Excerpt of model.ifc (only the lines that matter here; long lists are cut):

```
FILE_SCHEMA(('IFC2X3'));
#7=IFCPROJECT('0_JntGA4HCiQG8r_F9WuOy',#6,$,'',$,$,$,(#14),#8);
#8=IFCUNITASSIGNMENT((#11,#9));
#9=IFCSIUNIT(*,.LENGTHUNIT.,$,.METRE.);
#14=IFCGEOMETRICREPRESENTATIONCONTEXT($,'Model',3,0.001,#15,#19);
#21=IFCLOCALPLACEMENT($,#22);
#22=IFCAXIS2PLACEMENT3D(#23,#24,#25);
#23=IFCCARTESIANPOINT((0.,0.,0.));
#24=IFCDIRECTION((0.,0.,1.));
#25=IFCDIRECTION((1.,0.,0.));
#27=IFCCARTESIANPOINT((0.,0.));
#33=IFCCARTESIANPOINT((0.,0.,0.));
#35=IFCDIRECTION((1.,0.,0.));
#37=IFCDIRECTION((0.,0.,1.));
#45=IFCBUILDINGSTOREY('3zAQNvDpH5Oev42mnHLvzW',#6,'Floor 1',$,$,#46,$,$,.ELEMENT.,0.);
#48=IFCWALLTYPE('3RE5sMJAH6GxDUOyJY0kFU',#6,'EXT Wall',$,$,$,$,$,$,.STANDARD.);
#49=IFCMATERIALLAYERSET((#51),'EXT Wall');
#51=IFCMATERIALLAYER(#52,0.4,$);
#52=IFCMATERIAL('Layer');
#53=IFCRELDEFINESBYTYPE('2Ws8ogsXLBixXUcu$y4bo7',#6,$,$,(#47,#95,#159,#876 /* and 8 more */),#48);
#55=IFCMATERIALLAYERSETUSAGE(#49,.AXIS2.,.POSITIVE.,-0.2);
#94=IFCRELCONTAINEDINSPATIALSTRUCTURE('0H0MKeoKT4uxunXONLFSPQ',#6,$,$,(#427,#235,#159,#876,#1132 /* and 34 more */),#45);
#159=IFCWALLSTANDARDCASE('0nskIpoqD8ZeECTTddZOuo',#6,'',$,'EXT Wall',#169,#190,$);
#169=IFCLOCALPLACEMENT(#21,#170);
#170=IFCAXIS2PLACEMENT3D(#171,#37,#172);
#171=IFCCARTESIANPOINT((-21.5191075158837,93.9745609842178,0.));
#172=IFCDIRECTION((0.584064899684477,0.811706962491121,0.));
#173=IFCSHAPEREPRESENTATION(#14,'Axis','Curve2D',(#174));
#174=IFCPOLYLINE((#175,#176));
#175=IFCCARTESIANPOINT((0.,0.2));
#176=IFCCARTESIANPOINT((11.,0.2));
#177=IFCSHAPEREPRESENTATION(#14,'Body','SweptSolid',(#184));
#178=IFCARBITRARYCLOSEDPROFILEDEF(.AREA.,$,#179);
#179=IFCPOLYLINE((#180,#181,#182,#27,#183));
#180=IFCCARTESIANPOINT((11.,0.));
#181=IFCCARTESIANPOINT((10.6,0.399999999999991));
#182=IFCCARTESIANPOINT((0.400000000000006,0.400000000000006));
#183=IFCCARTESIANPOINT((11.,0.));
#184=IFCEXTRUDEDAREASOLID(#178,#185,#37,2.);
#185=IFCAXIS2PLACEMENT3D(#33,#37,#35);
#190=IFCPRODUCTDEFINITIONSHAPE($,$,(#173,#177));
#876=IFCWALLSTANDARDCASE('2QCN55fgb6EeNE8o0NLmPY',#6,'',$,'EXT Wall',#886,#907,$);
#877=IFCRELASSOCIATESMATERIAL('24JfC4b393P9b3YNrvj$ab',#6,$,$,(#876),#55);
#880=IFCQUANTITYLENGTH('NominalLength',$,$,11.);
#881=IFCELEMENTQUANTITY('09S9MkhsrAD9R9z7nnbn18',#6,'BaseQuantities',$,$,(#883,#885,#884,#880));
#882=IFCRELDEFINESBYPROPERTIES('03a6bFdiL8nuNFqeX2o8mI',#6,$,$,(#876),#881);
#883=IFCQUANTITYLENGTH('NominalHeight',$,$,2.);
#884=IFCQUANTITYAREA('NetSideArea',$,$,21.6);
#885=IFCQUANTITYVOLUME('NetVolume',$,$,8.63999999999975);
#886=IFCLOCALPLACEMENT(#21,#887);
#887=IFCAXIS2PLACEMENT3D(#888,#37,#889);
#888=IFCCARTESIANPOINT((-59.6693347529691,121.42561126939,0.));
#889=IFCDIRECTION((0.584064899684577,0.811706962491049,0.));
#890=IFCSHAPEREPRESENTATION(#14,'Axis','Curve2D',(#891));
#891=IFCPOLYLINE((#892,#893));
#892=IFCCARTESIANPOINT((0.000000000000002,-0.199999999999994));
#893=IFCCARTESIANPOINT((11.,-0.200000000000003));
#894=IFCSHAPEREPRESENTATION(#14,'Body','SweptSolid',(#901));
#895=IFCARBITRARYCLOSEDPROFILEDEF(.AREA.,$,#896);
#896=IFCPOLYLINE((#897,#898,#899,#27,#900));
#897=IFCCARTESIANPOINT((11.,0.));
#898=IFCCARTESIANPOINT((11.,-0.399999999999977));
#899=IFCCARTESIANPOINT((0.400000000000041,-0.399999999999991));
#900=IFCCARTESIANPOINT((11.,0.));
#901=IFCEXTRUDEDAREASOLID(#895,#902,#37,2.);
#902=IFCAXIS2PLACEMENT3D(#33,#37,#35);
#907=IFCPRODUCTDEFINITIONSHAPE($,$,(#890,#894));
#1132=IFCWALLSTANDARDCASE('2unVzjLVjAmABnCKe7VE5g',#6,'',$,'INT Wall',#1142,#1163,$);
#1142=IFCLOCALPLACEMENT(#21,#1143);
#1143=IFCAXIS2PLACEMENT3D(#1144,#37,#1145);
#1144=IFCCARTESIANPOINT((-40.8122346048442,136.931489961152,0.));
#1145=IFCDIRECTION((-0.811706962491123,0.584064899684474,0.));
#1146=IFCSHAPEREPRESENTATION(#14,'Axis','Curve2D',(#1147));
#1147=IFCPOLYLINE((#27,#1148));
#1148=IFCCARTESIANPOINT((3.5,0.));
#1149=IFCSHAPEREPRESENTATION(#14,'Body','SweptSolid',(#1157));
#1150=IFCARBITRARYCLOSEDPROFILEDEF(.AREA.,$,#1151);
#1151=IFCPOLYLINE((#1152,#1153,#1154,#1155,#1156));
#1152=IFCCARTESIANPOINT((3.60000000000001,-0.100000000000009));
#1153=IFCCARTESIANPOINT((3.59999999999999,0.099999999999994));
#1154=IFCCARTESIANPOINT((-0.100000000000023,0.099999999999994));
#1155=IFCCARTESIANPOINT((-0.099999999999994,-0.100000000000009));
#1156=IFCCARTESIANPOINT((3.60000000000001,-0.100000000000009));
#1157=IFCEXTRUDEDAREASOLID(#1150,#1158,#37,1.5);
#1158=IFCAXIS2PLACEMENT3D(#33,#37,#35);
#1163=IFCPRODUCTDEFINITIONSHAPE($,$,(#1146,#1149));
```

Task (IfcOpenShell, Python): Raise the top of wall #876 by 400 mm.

```python
import ifcopenshell
import ifcopenshell.api.pset
import ifcopenshell.geom
import ifcopenshell.util.element
import ifcopenshell.util.shape
import ifcopenshell.util.unit

model = ifcopenshell.open("model.ifc")
unit_scale = ifcopenshell.util.unit.calculate_unit_scale(model)
area_scale = ifcopenshell.util.unit.calculate_unit_scale(model, "AREAUNIT")
volume_scale = ifcopenshell.util.unit.calculate_unit_scale(model, "VOLUMEUNIT")
settings = ifcopenshell.geom.settings()


def volume(element):
    """Net volume in cubic metres, openings subtracted."""
    shape = ifcopenshell.geom.create_shape(settings, element)
    return ifcopenshell.util.shape.get_volume(shape.geometry)


wall = model.by_guid("2QCN55fgb6EeNE8o0NLmPY")
before = volume(wall)

body = next(r for r in wall.Representation.Representations if r.RepresentationIdentifier == "Body")
solid = body.Items[0]
old_height = solid.Depth
solid.Depth += 0.4 / unit_scale
after = volume(wall)
thickness = 0.4  # wall thickness in metres

# Update the stored height, areas and volumes.
qto = model.by_id(ifcopenshell.util.element.get_pset(wall, "BaseQuantities", should_inherit=False)["id"])
ifcopenshell.api.pset.edit_qto(model, qto=qto, properties={
    "NominalHeight": solid.Depth,
    "NetVolume": after / volume_scale,
    "NetSideArea": after / thickness / area_scale,
})

print(f"height {old_height:g} -> {solid.Depth:g}, volume {before:.3f} -> {after:.3f} m3")

model.write("model_updated.ifc")
```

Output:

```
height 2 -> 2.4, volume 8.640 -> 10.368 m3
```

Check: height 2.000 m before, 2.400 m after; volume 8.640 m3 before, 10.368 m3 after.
